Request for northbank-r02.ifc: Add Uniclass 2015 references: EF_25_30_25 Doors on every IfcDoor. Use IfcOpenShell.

First a look at what the model holds.

```python
import ifcopenshell

model = ifcopenshell.open("northbank-r02.ifc")
print(model.schema)
print("classifications:", [c.Name for c in model.by_type("IfcClassification")])
for ifc_class in ("IfcDoor", "IfcRoof", "IfcStair", "IfcWall", "IfcWindow"):
    print(ifc_class, len(model.by_type(ifc_class)))
```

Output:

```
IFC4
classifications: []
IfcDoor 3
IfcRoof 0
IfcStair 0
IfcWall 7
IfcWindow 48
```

```python
import ifcopenshell
import ifcopenshell.api.classification

model = ifcopenshell.open("northbank-r02.ifc")

system = ifcopenshell.api.classification.add_classification(model, classification="Uniclass 2015")

codes = {
    "IfcDoor": ("EF_25_30_25", "Doors"),
}
for ifc_class, (code, name) in codes.items():
    products = model.by_type(ifc_class)
    ifcopenshell.api.classification.add_reference(
        model, products=products, classification=system, identification=code, name=name
    )
    print(code, len(products))

model.write("northbank-r02_v2.ifc")
```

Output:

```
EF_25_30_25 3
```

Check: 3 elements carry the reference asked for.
